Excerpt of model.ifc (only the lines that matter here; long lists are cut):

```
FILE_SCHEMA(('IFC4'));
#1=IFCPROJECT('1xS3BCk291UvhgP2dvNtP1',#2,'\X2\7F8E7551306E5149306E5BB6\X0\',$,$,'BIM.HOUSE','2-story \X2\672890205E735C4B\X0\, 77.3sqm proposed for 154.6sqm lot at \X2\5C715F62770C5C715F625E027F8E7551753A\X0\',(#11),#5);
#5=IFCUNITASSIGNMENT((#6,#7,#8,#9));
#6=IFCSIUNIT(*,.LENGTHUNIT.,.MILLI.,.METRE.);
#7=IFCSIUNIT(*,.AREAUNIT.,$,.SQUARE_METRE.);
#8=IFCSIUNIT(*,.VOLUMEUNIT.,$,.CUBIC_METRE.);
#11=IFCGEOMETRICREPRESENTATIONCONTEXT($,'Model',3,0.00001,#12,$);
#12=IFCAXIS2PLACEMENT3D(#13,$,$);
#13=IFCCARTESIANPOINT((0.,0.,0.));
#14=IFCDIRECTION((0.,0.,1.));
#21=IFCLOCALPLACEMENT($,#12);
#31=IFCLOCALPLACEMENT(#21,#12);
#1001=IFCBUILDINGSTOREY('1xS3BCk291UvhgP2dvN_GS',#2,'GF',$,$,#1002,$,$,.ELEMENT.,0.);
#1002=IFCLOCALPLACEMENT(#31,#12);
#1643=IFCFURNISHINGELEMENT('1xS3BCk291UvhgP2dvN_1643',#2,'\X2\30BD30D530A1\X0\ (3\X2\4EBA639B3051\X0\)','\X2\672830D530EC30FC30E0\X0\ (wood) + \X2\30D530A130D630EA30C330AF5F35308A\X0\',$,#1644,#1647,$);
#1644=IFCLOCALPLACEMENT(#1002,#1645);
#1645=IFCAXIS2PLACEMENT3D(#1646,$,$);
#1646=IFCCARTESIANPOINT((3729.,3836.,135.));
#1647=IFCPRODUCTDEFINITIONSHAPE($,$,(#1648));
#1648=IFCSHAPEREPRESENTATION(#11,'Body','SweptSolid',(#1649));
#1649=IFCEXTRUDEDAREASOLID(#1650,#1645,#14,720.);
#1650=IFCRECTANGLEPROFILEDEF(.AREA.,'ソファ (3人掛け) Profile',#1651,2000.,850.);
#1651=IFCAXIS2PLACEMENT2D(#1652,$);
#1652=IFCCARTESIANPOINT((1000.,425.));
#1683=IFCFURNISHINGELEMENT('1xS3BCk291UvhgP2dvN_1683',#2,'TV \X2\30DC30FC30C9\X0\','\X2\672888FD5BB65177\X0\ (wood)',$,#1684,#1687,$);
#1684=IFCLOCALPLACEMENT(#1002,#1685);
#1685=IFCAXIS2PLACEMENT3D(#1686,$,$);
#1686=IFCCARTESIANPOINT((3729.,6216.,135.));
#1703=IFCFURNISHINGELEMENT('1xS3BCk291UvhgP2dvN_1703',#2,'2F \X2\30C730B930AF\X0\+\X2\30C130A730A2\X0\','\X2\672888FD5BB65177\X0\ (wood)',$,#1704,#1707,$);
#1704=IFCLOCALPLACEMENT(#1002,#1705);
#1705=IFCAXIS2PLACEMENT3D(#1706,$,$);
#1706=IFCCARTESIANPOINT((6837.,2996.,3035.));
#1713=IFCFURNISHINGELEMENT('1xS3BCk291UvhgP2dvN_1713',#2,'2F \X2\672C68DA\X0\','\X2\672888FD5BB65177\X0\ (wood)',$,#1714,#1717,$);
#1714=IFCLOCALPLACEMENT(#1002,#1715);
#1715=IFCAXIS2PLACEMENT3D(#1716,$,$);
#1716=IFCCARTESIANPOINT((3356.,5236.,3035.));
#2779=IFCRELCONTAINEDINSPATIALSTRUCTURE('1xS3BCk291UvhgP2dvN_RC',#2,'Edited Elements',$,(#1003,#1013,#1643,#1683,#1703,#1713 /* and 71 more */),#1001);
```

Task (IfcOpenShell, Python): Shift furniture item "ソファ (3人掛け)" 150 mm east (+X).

```python
import ifcopenshell
import ifcopenshell.api.geometry
import ifcopenshell.util.placement
import ifcopenshell.util.unit

model = ifcopenshell.open("model.ifc")
unit_scale = ifcopenshell.util.unit.calculate_unit_scale(model)

item = model.by_guid("1xS3BCk291UvhgP2dvN_1643")
matrix = ifcopenshell.util.placement.get_local_placement(item.ObjectPlacement)
matrix[0, 3] += 0.15 / unit_scale
ifcopenshell.api.geometry.edit_object_placement(model, product=item, matrix=matrix, is_si=False)

print(ifcopenshell.util.placement.get_local_placement(item.ObjectPlacement).round(3) + 0.0)

model.write("model_v2.ifc")
```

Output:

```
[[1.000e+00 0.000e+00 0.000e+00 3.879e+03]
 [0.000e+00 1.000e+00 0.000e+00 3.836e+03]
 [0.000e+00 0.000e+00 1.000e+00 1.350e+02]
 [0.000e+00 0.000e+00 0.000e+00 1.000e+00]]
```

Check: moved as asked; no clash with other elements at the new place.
